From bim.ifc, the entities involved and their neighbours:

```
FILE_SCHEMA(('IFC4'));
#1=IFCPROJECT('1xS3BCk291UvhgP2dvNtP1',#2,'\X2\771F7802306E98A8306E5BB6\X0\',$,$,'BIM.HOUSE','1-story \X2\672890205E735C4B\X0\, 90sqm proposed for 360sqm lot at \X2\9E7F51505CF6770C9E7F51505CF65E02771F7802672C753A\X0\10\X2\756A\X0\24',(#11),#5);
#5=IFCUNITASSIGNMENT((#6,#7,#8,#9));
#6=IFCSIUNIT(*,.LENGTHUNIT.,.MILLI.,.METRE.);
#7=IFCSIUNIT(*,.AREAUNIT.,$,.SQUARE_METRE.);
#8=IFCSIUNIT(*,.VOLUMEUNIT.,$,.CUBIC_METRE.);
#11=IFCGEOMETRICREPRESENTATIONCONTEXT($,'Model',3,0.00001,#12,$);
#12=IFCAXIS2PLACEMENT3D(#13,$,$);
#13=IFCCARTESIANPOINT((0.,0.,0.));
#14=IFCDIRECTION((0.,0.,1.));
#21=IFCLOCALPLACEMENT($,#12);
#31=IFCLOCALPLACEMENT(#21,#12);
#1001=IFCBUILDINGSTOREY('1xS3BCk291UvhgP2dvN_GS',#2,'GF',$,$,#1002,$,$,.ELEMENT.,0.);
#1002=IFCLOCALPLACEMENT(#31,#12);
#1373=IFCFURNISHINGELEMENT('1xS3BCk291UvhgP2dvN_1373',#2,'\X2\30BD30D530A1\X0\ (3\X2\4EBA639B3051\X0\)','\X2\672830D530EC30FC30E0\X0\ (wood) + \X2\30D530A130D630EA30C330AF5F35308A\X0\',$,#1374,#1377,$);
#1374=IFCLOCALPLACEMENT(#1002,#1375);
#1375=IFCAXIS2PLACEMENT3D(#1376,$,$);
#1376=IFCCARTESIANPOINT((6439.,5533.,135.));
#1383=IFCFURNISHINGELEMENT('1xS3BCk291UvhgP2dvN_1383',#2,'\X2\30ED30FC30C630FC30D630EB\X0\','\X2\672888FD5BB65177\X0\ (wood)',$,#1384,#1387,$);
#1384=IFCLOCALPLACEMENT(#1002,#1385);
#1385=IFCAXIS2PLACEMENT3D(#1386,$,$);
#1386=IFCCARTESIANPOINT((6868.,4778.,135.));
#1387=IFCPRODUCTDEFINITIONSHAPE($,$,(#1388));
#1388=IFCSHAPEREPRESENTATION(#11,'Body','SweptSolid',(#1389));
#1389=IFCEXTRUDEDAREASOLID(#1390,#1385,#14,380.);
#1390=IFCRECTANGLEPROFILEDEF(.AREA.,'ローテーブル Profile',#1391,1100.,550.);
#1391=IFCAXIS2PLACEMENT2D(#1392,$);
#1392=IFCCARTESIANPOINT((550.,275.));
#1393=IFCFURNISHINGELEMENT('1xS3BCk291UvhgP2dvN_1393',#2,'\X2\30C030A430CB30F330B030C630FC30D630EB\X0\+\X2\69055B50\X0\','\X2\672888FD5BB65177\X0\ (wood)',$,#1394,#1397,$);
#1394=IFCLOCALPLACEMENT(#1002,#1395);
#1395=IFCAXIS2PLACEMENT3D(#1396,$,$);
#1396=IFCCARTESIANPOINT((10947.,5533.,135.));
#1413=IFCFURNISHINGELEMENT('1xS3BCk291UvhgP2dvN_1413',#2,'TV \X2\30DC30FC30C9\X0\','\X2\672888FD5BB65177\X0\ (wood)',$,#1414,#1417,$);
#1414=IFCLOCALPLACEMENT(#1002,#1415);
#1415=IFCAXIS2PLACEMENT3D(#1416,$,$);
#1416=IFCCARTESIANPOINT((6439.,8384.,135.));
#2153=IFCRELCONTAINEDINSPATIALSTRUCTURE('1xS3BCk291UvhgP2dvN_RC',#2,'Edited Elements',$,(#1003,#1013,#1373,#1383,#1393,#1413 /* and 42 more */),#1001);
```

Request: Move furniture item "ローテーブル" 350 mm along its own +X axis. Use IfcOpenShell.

```python
import ifcopenshell
import ifcopenshell.api.geometry
import ifcopenshell.util.placement
import ifcopenshell.util.unit

model = ifcopenshell.open("bim.ifc")
unit_scale = ifcopenshell.util.unit.calculate_unit_scale(model)

item = model.by_id(1383)
matrix = ifcopenshell.util.placement.get_local_placement(item.ObjectPlacement)
matrix[:3, 3] += matrix[:3, 0] * 0.35 / unit_scale
ifcopenshell.api.geometry.edit_object_placement(model, product=item, matrix=matrix, is_si=False)

print(ifcopenshell.util.placement.get_local_placement(item.ObjectPlacement).round(3) + 0.0)

model.write("bim_v2.ifc")
```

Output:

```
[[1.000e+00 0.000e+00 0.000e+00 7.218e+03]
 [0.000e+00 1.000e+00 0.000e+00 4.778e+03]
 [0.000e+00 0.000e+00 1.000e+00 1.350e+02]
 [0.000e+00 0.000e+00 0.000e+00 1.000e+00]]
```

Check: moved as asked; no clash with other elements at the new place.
